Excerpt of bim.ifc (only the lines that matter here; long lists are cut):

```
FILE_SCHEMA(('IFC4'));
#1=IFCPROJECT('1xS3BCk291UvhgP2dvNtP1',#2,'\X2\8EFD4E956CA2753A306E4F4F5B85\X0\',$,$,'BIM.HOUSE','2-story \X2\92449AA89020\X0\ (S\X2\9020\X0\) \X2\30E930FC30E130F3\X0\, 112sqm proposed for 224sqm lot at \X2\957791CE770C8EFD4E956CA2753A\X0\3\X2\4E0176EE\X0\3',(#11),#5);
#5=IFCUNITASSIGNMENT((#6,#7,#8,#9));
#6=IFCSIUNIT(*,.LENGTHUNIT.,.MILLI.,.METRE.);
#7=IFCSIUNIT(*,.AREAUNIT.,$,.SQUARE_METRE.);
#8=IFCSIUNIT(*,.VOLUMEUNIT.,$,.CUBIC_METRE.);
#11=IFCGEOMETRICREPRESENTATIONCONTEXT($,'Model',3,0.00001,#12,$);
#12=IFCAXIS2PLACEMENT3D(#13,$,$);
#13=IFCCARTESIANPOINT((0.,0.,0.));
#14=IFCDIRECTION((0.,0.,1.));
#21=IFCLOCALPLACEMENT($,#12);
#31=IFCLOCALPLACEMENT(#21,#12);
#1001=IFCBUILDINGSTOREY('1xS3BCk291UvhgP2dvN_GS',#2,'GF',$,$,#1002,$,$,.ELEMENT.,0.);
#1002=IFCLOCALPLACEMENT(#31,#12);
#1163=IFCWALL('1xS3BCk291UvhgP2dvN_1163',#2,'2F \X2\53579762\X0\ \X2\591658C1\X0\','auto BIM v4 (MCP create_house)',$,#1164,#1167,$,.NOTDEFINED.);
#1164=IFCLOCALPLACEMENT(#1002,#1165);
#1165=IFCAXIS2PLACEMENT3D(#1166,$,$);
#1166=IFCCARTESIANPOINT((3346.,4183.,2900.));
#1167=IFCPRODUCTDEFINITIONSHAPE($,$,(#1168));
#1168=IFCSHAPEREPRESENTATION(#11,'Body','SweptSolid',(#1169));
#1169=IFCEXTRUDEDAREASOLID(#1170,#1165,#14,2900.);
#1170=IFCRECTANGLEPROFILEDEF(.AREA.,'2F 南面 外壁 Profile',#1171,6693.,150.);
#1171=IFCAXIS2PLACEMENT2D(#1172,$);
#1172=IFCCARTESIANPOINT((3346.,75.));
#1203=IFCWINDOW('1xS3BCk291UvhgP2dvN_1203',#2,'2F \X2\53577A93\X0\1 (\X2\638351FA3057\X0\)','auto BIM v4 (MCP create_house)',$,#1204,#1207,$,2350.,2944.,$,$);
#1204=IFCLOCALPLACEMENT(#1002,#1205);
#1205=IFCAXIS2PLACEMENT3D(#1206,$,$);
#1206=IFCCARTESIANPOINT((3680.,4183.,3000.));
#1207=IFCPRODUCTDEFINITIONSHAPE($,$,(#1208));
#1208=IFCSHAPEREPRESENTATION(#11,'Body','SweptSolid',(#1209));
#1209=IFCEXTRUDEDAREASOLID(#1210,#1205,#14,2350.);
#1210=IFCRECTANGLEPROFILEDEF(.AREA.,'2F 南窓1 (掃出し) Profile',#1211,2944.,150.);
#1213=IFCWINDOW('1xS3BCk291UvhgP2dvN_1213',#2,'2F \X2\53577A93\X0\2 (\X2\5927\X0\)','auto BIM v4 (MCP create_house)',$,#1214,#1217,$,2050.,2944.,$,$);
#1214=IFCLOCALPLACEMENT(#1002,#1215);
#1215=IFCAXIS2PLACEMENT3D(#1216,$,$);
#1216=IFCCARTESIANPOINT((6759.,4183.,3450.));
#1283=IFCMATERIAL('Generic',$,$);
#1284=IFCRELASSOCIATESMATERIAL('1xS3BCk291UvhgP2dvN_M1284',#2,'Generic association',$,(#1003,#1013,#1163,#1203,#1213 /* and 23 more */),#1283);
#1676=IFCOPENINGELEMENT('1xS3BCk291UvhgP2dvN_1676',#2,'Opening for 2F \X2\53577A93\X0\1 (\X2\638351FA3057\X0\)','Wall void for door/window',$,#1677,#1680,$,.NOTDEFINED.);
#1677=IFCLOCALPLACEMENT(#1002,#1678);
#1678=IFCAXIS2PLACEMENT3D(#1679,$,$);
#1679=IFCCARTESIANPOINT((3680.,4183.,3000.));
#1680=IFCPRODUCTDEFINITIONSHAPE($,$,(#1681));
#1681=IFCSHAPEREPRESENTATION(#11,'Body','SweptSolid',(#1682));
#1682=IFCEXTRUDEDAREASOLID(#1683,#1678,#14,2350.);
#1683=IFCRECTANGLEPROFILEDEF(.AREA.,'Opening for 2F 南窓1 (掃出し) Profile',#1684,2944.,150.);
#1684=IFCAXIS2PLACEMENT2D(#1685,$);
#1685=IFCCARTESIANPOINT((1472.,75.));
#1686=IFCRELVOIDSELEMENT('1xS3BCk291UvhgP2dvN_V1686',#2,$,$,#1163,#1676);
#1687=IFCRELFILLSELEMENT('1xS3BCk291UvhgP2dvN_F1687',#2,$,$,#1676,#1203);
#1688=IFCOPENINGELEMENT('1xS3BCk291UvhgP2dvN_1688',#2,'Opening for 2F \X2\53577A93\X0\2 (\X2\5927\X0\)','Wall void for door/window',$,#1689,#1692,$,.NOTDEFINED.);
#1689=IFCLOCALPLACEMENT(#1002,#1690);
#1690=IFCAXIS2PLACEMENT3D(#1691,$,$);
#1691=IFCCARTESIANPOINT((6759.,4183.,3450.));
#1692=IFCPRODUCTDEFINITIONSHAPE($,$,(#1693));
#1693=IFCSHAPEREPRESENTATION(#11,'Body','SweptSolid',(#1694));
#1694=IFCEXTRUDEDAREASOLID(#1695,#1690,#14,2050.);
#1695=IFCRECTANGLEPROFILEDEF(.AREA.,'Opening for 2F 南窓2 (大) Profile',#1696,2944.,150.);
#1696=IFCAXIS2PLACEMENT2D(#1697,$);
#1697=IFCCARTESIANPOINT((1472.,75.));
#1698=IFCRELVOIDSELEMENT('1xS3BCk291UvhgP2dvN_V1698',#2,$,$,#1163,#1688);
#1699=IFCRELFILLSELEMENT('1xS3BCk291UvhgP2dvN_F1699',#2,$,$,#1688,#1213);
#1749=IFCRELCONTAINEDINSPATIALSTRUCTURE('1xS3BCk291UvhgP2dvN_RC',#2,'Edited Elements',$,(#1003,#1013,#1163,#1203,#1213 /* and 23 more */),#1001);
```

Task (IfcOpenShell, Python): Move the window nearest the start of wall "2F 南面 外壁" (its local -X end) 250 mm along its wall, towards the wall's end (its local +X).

```python
import ifcopenshell
import ifcopenshell.api.geometry
import ifcopenshell.util.placement

model = ifcopenshell.open("bim.ifc")

window = model.by_id(1203)
opening = window.FillsVoids[0].RelatingOpeningElement
wall = opening.VoidsElements[0].RelatingBuildingElement

wall_matrix = ifcopenshell.util.placement.get_local_placement(wall.ObjectPlacement)
shift = wall_matrix[:3, 0] * 250.0
before = ifcopenshell.util.placement.get_local_placement(window.ObjectPlacement)[:3, 3].copy()

# The window is not placed relative to its opening, so move both.
for product in (opening, window):
    matrix = ifcopenshell.util.placement.get_local_placement(product.ObjectPlacement)
    matrix[:3, 3] += shift
    ifcopenshell.api.geometry.edit_object_placement(model, product=product, matrix=matrix, is_si=False)

after = ifcopenshell.util.placement.get_local_placement(window.ObjectPlacement)[:3, 3]
print("window moved by", (after - before).round(3) + 0.0)

model.write("bim_updated.ifc")
```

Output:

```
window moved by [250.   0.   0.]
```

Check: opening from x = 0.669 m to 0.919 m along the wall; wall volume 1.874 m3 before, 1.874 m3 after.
